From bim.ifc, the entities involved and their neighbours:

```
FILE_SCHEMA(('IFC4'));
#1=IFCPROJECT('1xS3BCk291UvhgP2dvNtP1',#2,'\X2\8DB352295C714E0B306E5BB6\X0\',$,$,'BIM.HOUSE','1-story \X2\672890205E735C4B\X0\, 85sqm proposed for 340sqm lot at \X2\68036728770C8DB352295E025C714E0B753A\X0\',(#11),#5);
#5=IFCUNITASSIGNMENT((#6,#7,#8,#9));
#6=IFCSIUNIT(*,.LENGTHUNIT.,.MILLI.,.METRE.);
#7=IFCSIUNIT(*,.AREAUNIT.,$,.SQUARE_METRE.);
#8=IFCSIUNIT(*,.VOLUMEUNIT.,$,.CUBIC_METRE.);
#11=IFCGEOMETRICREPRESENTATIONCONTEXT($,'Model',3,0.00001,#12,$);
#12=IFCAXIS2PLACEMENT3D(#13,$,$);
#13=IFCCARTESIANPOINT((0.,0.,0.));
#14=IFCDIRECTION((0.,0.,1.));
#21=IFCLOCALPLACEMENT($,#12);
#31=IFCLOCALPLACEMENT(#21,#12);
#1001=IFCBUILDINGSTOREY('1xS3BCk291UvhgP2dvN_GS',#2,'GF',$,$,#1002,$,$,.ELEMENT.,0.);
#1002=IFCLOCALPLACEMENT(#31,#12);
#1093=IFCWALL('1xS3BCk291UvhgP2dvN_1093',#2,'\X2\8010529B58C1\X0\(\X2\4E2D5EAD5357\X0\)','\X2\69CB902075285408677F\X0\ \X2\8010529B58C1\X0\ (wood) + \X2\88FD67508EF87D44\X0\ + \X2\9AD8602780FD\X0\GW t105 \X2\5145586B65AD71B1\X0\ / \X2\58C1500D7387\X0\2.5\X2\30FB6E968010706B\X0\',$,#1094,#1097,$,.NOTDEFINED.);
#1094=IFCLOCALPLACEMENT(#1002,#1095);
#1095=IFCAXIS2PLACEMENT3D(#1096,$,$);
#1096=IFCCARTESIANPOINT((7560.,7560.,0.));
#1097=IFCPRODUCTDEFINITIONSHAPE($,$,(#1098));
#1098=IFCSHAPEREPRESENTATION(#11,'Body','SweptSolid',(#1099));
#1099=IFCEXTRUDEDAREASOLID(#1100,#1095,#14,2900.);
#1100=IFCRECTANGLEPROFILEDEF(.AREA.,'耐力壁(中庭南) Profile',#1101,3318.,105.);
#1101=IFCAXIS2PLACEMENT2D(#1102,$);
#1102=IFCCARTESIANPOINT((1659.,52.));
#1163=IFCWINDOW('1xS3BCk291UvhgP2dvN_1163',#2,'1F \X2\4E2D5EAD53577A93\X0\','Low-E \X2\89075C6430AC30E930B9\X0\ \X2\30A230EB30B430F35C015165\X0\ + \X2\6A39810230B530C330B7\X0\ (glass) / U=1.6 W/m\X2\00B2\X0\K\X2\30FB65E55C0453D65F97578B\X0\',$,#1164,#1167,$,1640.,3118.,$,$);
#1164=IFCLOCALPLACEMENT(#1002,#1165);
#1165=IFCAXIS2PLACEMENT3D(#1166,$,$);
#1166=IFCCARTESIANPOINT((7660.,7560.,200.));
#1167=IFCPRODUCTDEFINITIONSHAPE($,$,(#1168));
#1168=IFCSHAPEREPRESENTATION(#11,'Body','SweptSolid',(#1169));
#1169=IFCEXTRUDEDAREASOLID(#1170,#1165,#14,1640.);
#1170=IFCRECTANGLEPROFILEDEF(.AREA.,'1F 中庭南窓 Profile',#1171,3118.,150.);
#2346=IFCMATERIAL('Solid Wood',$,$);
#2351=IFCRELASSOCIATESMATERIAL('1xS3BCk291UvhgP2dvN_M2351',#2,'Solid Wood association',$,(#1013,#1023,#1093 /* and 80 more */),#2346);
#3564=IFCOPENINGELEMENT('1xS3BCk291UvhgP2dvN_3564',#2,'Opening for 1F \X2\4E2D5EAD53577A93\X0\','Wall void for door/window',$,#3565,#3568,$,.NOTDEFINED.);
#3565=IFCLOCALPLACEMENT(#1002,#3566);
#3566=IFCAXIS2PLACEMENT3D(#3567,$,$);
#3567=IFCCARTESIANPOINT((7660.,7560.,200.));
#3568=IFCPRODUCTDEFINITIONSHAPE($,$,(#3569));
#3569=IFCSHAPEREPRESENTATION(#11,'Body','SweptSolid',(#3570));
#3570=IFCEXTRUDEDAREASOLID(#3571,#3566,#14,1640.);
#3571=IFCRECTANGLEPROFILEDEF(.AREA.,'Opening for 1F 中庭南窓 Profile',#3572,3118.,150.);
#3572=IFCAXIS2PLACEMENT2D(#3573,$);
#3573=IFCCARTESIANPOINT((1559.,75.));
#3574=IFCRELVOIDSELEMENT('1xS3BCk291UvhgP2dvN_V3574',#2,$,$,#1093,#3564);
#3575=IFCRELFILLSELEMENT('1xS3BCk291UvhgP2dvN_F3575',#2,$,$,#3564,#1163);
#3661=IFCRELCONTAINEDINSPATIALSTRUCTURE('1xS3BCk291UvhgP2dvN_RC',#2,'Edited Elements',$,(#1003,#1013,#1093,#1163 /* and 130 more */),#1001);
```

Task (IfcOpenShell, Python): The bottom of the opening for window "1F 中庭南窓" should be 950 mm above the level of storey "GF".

```python
import numpy as np
import ifcopenshell
import ifcopenshell.api.geometry
import ifcopenshell.geom
import ifcopenshell.util.element
import ifcopenshell.util.placement
import ifcopenshell.util.shape
import ifcopenshell.util.unit

model = ifcopenshell.open("bim.ifc")
unit_scale = ifcopenshell.util.unit.calculate_unit_scale(model)

window = model.by_id(1163)
opening = window.FillsVoids[0].RelatingOpeningElement
storey = ifcopenshell.util.element.get_container(window, ifc_class="IfcBuildingStorey")
level = ifcopenshell.util.placement.get_local_placement(storey.ObjectPlacement)[2, 3]

# The opening's origin need not be at the sill, so measure its lowest point.
shape = ifcopenshell.geom.create_shape(ifcopenshell.geom.settings(), opening)
bottom = ifcopenshell.util.shape.get_shape_bottom_elevation(shape, shape.geometry) / unit_scale
dz = level + 950.0 - bottom

shift = np.array([0.0, 0.0, dz])
# The window is not placed relative to its opening, so move both.
for product in (opening, window):
    matrix = ifcopenshell.util.placement.get_local_placement(product.ObjectPlacement)
    matrix[:3, 3] += shift
    ifcopenshell.api.geometry.edit_object_placement(model, product=product, matrix=matrix, is_si=False)

print(f"moved by {dz * unit_scale:+.3f} m")

model.write("bim_v2.ifc")
```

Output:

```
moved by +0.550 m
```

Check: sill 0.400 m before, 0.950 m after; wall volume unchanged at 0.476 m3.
